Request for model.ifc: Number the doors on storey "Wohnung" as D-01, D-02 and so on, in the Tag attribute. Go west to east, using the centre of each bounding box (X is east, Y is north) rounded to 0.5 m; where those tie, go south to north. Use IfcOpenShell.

First a look at what the model holds.

```python
import ifcopenshell
import ifcopenshell.util.element
import ifcopenshell.util.placement

model = ifcopenshell.open("model.ifc")
print(model.schema)
storey = next(s for s in model.by_type("IfcBuildingStorey") if s.Name == "Wohnung")
doors = [e for e in ifcopenshell.util.element.get_decomposition(storey) if e.is_a("IfcDoor")]
for e in sorted(doors, key=lambda e: e.id()):
    origin = ifcopenshell.util.placement.get_local_placement(e.ObjectPlacement)[:3, 3]
    print(e.id(), e.Tag, e.Name, origin.round(2) + 0.0, sep=" | ")
```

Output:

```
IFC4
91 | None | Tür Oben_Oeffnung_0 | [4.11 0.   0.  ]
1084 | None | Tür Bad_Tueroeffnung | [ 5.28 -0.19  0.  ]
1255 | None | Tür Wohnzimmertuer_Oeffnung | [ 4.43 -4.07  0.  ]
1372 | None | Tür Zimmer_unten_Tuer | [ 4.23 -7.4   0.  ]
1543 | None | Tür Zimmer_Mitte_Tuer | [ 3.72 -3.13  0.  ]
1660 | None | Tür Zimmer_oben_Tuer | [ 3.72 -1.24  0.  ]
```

```python
import ifcopenshell
import ifcopenshell.geom
import ifcopenshell.util.element
import ifcopenshell.util.shape

model = ifcopenshell.open("model.ifc")
settings = ifcopenshell.geom.settings()
settings.set("use-world-coords", True)


def centre(element):
    shape = ifcopenshell.geom.create_shape(settings, element)
    return ifcopenshell.util.shape.get_bbox_centroid(shape.geometry)


storey = next(s for s in model.by_type("IfcBuildingStorey") if s.Name == "Wohnung")
doors = [e for e in ifcopenshell.util.element.get_decomposition(storey) if e.is_a("IfcDoor")]

# Insertion points can sit at a corner or the storey origin, so sort by the geometry (in metres).
centres = {e: centre(e) for e in doors}
doors.sort(key=lambda e: (round(centres[e][0] / 0.5), centres[e][1]))

for i, e in enumerate(doors, start=1):
    number = f"D-{i:02d}"
    e.Tag = number
    print(e.id(), number)

model.write("model_edited.ifc")
```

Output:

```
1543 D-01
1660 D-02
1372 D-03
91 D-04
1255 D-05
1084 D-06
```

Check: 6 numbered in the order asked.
